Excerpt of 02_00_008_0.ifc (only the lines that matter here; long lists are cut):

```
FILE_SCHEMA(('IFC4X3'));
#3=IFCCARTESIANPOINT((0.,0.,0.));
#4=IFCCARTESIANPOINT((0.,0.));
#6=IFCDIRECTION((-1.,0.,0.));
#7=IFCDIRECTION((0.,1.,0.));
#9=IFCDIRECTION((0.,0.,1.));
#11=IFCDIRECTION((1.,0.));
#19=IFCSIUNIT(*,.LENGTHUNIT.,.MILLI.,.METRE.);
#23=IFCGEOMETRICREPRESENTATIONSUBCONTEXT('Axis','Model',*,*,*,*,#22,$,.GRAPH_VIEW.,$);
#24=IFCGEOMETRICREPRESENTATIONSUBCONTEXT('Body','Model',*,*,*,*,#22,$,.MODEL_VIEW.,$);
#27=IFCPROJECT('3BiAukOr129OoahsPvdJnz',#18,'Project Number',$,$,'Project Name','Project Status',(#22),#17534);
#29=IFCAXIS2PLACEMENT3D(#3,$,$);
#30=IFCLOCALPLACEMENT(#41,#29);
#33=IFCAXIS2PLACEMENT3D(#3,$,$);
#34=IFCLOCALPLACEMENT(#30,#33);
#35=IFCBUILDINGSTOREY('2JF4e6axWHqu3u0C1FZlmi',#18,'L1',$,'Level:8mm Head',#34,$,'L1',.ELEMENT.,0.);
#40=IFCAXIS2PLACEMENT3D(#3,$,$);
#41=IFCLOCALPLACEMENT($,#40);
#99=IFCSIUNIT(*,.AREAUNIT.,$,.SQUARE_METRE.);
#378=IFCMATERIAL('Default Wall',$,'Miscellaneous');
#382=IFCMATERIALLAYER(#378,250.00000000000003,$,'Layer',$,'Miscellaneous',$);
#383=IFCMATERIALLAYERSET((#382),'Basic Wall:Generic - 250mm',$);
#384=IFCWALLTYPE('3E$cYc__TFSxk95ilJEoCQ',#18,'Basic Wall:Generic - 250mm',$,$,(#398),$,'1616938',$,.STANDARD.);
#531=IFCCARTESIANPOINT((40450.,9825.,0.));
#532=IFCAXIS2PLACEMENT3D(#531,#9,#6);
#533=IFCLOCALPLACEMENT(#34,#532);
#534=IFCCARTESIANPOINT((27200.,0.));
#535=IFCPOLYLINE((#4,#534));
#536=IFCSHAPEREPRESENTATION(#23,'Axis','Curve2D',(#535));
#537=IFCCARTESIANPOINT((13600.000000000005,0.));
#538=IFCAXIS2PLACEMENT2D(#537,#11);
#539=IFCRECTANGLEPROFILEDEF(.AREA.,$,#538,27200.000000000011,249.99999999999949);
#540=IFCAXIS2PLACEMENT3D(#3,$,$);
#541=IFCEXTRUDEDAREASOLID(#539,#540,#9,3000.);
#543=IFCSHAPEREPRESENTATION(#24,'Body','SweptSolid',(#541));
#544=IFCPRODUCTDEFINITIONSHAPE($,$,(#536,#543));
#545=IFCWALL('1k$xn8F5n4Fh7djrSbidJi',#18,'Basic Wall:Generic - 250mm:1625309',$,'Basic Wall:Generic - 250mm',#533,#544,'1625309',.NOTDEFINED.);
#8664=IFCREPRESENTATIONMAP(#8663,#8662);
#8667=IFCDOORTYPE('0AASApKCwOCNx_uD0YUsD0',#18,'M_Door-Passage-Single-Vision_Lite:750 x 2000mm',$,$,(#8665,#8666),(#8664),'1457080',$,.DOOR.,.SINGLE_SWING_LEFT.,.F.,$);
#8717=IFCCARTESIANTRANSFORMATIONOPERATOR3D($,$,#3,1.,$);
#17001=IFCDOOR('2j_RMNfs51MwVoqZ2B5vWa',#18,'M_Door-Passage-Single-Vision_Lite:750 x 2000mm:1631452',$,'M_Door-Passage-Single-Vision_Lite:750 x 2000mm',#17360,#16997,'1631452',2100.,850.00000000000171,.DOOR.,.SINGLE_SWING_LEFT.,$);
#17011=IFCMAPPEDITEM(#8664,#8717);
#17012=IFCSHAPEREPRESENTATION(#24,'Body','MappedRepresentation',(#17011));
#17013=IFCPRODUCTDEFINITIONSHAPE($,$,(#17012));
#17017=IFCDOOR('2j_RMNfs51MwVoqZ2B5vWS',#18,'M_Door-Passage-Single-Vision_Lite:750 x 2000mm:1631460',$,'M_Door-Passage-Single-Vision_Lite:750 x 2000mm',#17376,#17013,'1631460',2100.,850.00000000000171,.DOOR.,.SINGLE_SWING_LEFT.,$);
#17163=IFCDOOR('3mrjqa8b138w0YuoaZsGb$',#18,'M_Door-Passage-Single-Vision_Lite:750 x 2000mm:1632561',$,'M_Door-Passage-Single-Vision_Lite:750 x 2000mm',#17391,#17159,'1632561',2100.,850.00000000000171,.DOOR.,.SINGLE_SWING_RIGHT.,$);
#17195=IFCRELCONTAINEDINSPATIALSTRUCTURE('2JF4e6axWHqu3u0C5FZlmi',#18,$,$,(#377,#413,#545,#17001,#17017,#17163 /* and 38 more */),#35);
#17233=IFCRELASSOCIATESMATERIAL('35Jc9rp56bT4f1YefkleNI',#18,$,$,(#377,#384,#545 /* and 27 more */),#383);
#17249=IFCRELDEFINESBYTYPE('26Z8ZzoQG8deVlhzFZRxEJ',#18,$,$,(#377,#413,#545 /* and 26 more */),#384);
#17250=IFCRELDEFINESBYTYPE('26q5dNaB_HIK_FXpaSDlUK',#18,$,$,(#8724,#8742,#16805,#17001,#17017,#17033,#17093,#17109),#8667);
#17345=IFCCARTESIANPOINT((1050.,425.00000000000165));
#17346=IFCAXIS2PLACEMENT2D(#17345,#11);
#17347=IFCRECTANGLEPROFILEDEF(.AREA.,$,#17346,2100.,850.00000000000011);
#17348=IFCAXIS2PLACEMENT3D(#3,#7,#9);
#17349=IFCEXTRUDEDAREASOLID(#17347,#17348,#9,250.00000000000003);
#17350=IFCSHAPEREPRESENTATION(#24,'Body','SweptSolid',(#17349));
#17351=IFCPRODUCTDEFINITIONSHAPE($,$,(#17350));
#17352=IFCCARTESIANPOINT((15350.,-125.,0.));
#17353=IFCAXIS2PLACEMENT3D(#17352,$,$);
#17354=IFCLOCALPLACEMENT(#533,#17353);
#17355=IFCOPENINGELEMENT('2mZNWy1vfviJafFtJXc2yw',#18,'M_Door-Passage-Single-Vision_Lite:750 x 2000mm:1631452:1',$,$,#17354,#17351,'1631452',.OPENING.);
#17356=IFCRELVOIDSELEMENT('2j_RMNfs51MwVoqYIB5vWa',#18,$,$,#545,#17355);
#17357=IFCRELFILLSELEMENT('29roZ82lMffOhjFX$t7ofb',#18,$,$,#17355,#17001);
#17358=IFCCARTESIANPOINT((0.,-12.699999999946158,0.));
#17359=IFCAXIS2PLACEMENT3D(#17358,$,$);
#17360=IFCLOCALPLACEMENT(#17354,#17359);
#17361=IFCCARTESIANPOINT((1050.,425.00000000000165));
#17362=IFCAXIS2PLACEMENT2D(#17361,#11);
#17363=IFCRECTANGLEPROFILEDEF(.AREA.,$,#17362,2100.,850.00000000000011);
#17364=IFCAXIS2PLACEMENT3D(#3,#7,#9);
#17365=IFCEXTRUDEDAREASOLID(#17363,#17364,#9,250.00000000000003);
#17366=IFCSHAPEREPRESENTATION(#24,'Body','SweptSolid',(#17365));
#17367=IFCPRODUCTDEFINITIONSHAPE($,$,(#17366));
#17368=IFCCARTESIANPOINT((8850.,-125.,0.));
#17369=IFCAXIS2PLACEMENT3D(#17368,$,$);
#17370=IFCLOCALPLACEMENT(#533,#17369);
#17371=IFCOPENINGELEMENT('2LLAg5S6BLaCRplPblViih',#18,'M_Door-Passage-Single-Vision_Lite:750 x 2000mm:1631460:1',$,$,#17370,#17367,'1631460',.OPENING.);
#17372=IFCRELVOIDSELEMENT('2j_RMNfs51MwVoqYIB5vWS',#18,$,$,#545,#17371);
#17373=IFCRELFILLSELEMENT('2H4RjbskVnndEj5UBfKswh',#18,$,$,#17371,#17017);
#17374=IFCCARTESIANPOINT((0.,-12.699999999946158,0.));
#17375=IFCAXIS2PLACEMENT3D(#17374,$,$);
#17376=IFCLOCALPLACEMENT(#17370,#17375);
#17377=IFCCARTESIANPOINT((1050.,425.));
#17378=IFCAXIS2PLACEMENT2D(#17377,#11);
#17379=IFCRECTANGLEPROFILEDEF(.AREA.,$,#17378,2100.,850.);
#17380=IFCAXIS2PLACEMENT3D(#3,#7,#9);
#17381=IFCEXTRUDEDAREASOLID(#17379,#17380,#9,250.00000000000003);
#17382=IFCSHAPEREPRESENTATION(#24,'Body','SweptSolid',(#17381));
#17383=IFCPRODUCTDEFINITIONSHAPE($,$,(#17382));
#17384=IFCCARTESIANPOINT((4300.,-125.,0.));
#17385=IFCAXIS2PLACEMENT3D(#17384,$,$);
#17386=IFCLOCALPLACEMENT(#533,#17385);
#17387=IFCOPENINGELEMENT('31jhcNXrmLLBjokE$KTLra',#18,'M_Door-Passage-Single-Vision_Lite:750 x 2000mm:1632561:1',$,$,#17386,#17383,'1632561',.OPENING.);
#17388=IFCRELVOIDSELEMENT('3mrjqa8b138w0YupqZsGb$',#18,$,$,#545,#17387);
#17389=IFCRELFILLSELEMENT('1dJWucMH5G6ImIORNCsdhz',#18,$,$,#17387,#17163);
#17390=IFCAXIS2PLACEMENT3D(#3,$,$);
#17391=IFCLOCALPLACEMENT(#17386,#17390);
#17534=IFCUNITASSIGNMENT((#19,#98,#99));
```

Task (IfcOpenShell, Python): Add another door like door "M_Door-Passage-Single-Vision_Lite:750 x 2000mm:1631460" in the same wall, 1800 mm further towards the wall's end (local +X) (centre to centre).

```python
import ifcopenshell
import ifcopenshell.api.feature
import ifcopenshell.api.geometry
import ifcopenshell.api.root
import ifcopenshell.geom
import ifcopenshell.util.element
import ifcopenshell.util.placement
import ifcopenshell.util.shape
import ifcopenshell.util.unit

model = ifcopenshell.open("02_00_008_0.ifc")
unit_scale = ifcopenshell.util.unit.calculate_unit_scale(model)
settings = ifcopenshell.geom.settings()


def volume(element):
    """Net volume in cubic metres, openings subtracted."""
    shape = ifcopenshell.geom.create_shape(settings, element)
    return ifcopenshell.util.shape.get_volume(shape.geometry)


def reuse_history(source, copy):
    """copy_class also copies each property set's owner history, people and application; keep the originals."""
    for rel in copy.IsDefinedBy:
        if rel.is_a("IfcRelDefinesByProperties") and (history := rel.RelatingPropertyDefinition.OwnerHistory):
            rel.RelatingPropertyDefinition.OwnerHistory = source.OwnerHistory
            ifcopenshell.util.element.remove_deep2(model, history)


door = model.by_guid("2j_RMNfs51MwVoqZ2B5vWS")
opening = door.FillsVoids[0].RelatingOpeningElement
wall = opening.VoidsElements[0].RelatingBuildingElement
before = volume(wall)
shift = ifcopenshell.util.placement.get_local_placement(wall.ObjectPlacement)[:3, 0] * 1.8 / unit_scale

# copy_class copies the void relationship, type, container and properties, but no geometry.
new_opening = ifcopenshell.api.root.copy_class(model, product=opening)
new_opening.Representation = ifcopenshell.util.element.copy_deep(
    model, opening.Representation, exclude=["IfcGeometricRepresentationContext", "IfcRepresentationMap"]
)
new_opening.Name = "M_Door-Passage-Single-Vision_Lite:750 x 2000mm"
new_opening.Tag = None
new_door = ifcopenshell.api.root.copy_class(model, product=door)
new_door.Representation = ifcopenshell.util.element.copy_deep(
    model, door.Representation, exclude=["IfcGeometricRepresentationContext", "IfcRepresentationMap"]
)
new_door.Name = "M_Door-Passage-Single-Vision_Lite:750 x 2000mm"
new_door.Tag = None
reuse_history(door, new_door)
ifcopenshell.api.feature.add_filling(model, opening=new_opening, element=new_door)

for old, new in ((opening, new_opening), (door, new_door)):
    matrix = ifcopenshell.util.placement.get_local_placement(old.ObjectPlacement)
    matrix[:3, 3] += shift
    ifcopenshell.api.geometry.edit_object_placement(model, product=new, matrix=matrix, is_si=False)

after = volume(wall)

print(f"wall volume {before:.3f} -> {after:.3f} m3")

model.write("02_00_008_0_edited.ifc")
```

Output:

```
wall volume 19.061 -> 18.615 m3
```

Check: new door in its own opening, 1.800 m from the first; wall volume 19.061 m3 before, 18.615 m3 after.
